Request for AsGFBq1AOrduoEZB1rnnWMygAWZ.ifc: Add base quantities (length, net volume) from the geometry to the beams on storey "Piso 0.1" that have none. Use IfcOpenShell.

First a look at what the model holds.

```python
import ifcopenshell
import ifcopenshell.util.element
import ifcopenshell.util.unit

model = ifcopenshell.open("AsGFBq1AOrduoEZB1rnnWMygAWZ.ifc")
print(model.schema)
for unit_type in ("LENGTHUNIT", "AREAUNIT", "VOLUMEUNIT"):
    print(unit_type, ifcopenshell.util.unit.calculate_unit_scale(model, unit_type))
storey = next(s for s in model.by_type("IfcBuildingStorey") if s.Name == "Piso 0.1")
beams = [e for e in ifcopenshell.util.element.get_decomposition(storey) if e.is_a("IfcBeam")]
for e in sorted(beams, key=lambda e: e.id()):
    print(e.id(), e.is_a(), e.Name, list(ifcopenshell.util.element.get_psets(e, qtos_only=True)), sep=" | ")
```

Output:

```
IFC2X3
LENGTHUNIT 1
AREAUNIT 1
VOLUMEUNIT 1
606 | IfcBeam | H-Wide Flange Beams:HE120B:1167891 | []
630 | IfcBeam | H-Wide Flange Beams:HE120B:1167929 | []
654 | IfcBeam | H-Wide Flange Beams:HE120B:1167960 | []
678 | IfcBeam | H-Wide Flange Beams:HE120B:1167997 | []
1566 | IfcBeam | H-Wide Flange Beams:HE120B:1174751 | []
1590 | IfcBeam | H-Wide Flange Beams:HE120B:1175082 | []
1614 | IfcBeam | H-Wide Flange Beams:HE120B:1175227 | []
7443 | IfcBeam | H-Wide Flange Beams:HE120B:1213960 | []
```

```python
import ifcopenshell
import ifcopenshell.api.pset
import ifcopenshell.geom
import ifcopenshell.util.element
import ifcopenshell.util.shape
import ifcopenshell.util.unit

model = ifcopenshell.open("AsGFBq1AOrduoEZB1rnnWMygAWZ.ifc")
unit_scale = ifcopenshell.util.unit.calculate_unit_scale(model)
volume_scale = ifcopenshell.util.unit.calculate_unit_scale(model, "VOLUMEUNIT")
settings = ifcopenshell.geom.settings()

storey = next(s for s in model.by_type("IfcBuildingStorey") if s.Name == "Piso 0.1")
beams = [e for e in ifcopenshell.util.element.get_decomposition(storey) if e.is_a("IfcBeam")]

for e in sorted(beams, key=lambda e: e.id()):
    if ifcopenshell.util.element.get_psets(e, qtos_only=True, should_inherit=False):
        continue
    # Geometry comes back in metres, in the element's own axes.
    shape = ifcopenshell.geom.create_shape(settings, e)
    values = {
        "Length": ifcopenshell.util.shape.get_max_xyz(shape.geometry) / unit_scale,
        "NetVolume": ifcopenshell.util.shape.get_volume(shape.geometry) / volume_scale,
    }
    qto = ifcopenshell.api.pset.add_qto(model, product=e, name="BaseQuantities")
    ifcopenshell.api.pset.edit_qto(model, qto=qto, properties=values)
    print(e.id(), {k: round(v, 3) for k, v in values.items()})

model.write("AsGFBq1AOrduoEZB1rnnWMygAWZ_updated.ifc")
```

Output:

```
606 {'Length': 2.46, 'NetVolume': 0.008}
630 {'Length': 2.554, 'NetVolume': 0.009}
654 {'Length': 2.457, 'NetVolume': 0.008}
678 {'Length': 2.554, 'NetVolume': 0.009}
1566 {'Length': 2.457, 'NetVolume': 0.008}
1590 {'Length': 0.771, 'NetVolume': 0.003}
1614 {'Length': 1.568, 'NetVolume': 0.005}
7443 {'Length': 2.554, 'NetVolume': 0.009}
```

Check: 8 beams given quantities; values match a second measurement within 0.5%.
